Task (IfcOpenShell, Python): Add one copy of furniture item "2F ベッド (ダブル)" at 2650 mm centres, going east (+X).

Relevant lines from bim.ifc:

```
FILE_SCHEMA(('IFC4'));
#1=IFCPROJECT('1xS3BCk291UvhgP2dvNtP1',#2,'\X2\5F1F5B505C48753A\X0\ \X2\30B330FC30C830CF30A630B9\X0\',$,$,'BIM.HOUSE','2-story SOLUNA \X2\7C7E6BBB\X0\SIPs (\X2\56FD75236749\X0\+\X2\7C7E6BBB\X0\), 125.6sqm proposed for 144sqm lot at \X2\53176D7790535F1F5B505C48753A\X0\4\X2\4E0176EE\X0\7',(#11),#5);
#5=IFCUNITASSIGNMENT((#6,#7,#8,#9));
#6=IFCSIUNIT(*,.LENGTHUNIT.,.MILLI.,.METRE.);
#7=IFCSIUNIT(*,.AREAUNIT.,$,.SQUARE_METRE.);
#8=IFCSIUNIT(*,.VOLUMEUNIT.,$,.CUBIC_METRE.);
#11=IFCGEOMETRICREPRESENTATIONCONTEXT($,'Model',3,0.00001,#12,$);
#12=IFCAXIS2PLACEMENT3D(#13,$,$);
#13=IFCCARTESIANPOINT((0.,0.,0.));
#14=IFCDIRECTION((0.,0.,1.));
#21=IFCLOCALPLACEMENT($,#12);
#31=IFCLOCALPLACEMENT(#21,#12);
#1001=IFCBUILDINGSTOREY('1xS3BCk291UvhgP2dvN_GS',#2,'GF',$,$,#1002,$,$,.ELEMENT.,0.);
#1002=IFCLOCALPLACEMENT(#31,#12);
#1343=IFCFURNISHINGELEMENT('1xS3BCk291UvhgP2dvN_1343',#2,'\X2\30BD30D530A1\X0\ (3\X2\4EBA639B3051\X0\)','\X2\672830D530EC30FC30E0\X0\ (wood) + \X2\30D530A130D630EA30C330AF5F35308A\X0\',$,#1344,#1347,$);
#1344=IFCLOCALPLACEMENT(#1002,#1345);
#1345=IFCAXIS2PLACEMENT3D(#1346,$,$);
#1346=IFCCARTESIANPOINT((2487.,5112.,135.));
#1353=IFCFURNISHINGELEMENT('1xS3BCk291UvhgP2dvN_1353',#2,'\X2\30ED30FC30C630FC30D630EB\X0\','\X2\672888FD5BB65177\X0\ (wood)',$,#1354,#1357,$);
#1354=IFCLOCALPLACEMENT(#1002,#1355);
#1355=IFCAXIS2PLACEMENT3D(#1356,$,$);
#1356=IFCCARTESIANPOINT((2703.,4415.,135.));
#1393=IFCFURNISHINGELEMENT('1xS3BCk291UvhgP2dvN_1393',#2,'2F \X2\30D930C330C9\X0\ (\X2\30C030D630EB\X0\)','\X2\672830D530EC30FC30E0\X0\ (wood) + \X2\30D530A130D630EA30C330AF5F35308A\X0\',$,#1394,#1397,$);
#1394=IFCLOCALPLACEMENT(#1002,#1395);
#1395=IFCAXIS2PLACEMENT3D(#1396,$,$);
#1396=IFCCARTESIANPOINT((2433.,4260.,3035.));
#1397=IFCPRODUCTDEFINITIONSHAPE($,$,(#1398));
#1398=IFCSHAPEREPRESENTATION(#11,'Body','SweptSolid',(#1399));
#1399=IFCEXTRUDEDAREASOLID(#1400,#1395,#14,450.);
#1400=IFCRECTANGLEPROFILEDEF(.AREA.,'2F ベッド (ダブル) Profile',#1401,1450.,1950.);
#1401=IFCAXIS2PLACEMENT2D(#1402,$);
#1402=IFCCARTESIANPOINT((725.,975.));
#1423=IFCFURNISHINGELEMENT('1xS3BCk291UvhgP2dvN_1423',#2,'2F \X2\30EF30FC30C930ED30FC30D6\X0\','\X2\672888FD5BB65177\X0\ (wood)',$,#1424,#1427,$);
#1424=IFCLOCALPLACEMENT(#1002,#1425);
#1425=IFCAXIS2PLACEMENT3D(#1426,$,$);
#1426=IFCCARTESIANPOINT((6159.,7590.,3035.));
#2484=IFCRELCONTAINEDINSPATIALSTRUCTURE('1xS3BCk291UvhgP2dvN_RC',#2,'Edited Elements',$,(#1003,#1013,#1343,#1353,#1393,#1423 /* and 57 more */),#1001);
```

```python
import numpy as np
import ifcopenshell
import ifcopenshell.api.geometry
import ifcopenshell.api.root
import ifcopenshell.util.element
import ifcopenshell.util.placement
import ifcopenshell.util.unit

model = ifcopenshell.open("bim.ifc")
unit_scale = ifcopenshell.util.unit.calculate_unit_scale(model)


def reuse_history(source, copy):
    """copy_class also copies each property set's owner history, people and application; keep the originals."""
    for rel in copy.IsDefinedBy:
        if rel.is_a("IfcRelDefinesByProperties") and (history := rel.RelatingPropertyDefinition.OwnerHistory):
            rel.RelatingPropertyDefinition.OwnerHistory = source.OwnerHistory
            ifcopenshell.util.element.remove_deep2(model, history)


source = model.by_guid("1xS3BCk291UvhgP2dvN_1393")
base = ifcopenshell.util.placement.get_local_placement(source.ObjectPlacement)
step = np.array([1.0, 0.0, 0.0]) * 2.65 / unit_scale

for i in range(1, 2):
    copy = ifcopenshell.api.root.copy_class(model, product=source)
    copy.Representation = ifcopenshell.util.element.copy_deep(
        model, source.Representation, exclude=["IfcGeometricRepresentationContext", "IfcRepresentationMap"]
    )
    reuse_history(source, copy)
    matrix = base.copy()
    matrix[:3, 3] += i * step
    print("added at", matrix[:3, 3].round(3) + 0.0)
    ifcopenshell.api.geometry.edit_object_placement(model, product=copy, matrix=matrix, is_si=False)

model.write("bim-out.ifc")
```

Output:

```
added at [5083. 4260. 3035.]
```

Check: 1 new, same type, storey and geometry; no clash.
